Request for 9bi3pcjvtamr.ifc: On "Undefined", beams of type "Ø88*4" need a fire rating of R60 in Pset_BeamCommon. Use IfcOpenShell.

First a look at what the model holds.

```python
import ifcopenshell
import ifcopenshell.util.element

model = ifcopenshell.open("9bi3pcjvtamr.ifc")
print(model.schema)
storey = next(s for s in model.by_type("IfcBuildingStorey") if s.Name == "Undefined")
beams = [e for e in ifcopenshell.util.element.get_decomposition(storey) if e.is_a("IfcBeam")]
seen = {}
for e in beams:
    element_type = ifcopenshell.util.element.get_type(e)
    key = (element_type.Name if element_type != e and element_type else None, ifcopenshell.util.element.get_pset(e, "Pset_BeamCommon", "FireRating"))
    seen[key] = seen.get(key, 0) + 1
for (name, value), count in sorted(seen.items(), key=str):
    print(count, "x", name, "|", value)
```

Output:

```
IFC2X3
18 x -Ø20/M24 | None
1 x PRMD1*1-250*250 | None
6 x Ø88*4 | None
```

```python
import ifcopenshell
import ifcopenshell.api.pset
import ifcopenshell.util.element

model = ifcopenshell.open("9bi3pcjvtamr.ifc")

storey = next(s for s in model.by_type("IfcBuildingStorey") if s.Name == "Undefined")
beams = [e for e in ifcopenshell.util.element.get_decomposition(storey) if e.is_a("IfcBeam")]

count = 0
for e in beams:
    element_type = ifcopenshell.util.element.get_type(e)
    if element_type in (None, e) or element_type.Name != "Ø88*4":
        continue
    found = ifcopenshell.util.element.get_pset(e, "Pset_BeamCommon", should_inherit=False)
    if found:
        pset = model.by_id(found["id"])
        if len(ifcopenshell.util.element.get_elements_by_pset(pset)) > 1:
            pset = ifcopenshell.api.pset.unshare_pset(model, products=[e], pset=pset)[0]
    else:
        pset = ifcopenshell.api.pset.add_pset(model, product=e, name="Pset_BeamCommon")
    ifcopenshell.api.pset.edit_pset(model, pset=pset, properties={"FireRating": "R60"})
    count += 1

print(count, "beams updated")

model.write("9bi3pcjvtamr-out.ifc")
```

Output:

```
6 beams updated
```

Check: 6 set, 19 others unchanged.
